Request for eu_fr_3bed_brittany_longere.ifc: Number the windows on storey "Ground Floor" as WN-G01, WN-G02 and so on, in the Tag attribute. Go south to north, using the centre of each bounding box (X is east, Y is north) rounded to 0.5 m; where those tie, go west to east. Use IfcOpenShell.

First a look at what the model holds.

```python
import ifcopenshell
import ifcopenshell.util.element
import ifcopenshell.util.placement

model = ifcopenshell.open("eu_fr_3bed_brittany_longere.ifc")
print(model.schema)
storey = next(s for s in model.by_type("IfcBuildingStorey") if s.Name == "Ground Floor")
windows = [e for e in ifcopenshell.util.element.get_decomposition(storey) if e.is_a("IfcWindow")]
for e in sorted(windows, key=lambda e: e.id()):
    origin = ifcopenshell.util.placement.get_local_placement(e.ObjectPlacement)[:3, 3]
    print(e.id(), e.Tag, e.Name, origin.round(2) + 0.0, sep=" | ")
```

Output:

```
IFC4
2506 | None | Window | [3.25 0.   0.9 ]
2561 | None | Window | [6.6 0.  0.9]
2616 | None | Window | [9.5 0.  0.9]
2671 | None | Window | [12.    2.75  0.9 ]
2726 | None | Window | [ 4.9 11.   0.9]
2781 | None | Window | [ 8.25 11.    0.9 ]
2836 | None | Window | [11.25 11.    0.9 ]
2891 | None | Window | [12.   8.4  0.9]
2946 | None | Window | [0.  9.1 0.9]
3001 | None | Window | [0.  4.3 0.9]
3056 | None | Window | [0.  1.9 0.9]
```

```python
import ifcopenshell
import ifcopenshell.geom
import ifcopenshell.util.element
import ifcopenshell.util.shape

model = ifcopenshell.open("eu_fr_3bed_brittany_longere.ifc")
settings = ifcopenshell.geom.settings()
settings.set("use-world-coords", True)


def centre(element):
    shape = ifcopenshell.geom.create_shape(settings, element)
    return ifcopenshell.util.shape.get_bbox_centroid(shape.geometry)


storey = next(s for s in model.by_type("IfcBuildingStorey") if s.Name == "Ground Floor")
windows = [e for e in ifcopenshell.util.element.get_decomposition(storey) if e.is_a("IfcWindow")]

# Insertion points can sit at a corner or the storey origin, so sort by the geometry (in metres).
centres = {e: centre(e) for e in windows}
windows.sort(key=lambda e: (round(centres[e][1] / 0.5), centres[e][0]))

for i, e in enumerate(windows, start=1):
    number = f"WN-G{i:02d}"
    e.Tag = number
    print(e.id(), number)

model.write("eu_fr_3bed_brittany_longere-out.ifc")
```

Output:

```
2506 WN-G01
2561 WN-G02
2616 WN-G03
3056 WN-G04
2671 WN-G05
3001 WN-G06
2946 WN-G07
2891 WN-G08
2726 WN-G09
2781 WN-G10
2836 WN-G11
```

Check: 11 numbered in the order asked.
